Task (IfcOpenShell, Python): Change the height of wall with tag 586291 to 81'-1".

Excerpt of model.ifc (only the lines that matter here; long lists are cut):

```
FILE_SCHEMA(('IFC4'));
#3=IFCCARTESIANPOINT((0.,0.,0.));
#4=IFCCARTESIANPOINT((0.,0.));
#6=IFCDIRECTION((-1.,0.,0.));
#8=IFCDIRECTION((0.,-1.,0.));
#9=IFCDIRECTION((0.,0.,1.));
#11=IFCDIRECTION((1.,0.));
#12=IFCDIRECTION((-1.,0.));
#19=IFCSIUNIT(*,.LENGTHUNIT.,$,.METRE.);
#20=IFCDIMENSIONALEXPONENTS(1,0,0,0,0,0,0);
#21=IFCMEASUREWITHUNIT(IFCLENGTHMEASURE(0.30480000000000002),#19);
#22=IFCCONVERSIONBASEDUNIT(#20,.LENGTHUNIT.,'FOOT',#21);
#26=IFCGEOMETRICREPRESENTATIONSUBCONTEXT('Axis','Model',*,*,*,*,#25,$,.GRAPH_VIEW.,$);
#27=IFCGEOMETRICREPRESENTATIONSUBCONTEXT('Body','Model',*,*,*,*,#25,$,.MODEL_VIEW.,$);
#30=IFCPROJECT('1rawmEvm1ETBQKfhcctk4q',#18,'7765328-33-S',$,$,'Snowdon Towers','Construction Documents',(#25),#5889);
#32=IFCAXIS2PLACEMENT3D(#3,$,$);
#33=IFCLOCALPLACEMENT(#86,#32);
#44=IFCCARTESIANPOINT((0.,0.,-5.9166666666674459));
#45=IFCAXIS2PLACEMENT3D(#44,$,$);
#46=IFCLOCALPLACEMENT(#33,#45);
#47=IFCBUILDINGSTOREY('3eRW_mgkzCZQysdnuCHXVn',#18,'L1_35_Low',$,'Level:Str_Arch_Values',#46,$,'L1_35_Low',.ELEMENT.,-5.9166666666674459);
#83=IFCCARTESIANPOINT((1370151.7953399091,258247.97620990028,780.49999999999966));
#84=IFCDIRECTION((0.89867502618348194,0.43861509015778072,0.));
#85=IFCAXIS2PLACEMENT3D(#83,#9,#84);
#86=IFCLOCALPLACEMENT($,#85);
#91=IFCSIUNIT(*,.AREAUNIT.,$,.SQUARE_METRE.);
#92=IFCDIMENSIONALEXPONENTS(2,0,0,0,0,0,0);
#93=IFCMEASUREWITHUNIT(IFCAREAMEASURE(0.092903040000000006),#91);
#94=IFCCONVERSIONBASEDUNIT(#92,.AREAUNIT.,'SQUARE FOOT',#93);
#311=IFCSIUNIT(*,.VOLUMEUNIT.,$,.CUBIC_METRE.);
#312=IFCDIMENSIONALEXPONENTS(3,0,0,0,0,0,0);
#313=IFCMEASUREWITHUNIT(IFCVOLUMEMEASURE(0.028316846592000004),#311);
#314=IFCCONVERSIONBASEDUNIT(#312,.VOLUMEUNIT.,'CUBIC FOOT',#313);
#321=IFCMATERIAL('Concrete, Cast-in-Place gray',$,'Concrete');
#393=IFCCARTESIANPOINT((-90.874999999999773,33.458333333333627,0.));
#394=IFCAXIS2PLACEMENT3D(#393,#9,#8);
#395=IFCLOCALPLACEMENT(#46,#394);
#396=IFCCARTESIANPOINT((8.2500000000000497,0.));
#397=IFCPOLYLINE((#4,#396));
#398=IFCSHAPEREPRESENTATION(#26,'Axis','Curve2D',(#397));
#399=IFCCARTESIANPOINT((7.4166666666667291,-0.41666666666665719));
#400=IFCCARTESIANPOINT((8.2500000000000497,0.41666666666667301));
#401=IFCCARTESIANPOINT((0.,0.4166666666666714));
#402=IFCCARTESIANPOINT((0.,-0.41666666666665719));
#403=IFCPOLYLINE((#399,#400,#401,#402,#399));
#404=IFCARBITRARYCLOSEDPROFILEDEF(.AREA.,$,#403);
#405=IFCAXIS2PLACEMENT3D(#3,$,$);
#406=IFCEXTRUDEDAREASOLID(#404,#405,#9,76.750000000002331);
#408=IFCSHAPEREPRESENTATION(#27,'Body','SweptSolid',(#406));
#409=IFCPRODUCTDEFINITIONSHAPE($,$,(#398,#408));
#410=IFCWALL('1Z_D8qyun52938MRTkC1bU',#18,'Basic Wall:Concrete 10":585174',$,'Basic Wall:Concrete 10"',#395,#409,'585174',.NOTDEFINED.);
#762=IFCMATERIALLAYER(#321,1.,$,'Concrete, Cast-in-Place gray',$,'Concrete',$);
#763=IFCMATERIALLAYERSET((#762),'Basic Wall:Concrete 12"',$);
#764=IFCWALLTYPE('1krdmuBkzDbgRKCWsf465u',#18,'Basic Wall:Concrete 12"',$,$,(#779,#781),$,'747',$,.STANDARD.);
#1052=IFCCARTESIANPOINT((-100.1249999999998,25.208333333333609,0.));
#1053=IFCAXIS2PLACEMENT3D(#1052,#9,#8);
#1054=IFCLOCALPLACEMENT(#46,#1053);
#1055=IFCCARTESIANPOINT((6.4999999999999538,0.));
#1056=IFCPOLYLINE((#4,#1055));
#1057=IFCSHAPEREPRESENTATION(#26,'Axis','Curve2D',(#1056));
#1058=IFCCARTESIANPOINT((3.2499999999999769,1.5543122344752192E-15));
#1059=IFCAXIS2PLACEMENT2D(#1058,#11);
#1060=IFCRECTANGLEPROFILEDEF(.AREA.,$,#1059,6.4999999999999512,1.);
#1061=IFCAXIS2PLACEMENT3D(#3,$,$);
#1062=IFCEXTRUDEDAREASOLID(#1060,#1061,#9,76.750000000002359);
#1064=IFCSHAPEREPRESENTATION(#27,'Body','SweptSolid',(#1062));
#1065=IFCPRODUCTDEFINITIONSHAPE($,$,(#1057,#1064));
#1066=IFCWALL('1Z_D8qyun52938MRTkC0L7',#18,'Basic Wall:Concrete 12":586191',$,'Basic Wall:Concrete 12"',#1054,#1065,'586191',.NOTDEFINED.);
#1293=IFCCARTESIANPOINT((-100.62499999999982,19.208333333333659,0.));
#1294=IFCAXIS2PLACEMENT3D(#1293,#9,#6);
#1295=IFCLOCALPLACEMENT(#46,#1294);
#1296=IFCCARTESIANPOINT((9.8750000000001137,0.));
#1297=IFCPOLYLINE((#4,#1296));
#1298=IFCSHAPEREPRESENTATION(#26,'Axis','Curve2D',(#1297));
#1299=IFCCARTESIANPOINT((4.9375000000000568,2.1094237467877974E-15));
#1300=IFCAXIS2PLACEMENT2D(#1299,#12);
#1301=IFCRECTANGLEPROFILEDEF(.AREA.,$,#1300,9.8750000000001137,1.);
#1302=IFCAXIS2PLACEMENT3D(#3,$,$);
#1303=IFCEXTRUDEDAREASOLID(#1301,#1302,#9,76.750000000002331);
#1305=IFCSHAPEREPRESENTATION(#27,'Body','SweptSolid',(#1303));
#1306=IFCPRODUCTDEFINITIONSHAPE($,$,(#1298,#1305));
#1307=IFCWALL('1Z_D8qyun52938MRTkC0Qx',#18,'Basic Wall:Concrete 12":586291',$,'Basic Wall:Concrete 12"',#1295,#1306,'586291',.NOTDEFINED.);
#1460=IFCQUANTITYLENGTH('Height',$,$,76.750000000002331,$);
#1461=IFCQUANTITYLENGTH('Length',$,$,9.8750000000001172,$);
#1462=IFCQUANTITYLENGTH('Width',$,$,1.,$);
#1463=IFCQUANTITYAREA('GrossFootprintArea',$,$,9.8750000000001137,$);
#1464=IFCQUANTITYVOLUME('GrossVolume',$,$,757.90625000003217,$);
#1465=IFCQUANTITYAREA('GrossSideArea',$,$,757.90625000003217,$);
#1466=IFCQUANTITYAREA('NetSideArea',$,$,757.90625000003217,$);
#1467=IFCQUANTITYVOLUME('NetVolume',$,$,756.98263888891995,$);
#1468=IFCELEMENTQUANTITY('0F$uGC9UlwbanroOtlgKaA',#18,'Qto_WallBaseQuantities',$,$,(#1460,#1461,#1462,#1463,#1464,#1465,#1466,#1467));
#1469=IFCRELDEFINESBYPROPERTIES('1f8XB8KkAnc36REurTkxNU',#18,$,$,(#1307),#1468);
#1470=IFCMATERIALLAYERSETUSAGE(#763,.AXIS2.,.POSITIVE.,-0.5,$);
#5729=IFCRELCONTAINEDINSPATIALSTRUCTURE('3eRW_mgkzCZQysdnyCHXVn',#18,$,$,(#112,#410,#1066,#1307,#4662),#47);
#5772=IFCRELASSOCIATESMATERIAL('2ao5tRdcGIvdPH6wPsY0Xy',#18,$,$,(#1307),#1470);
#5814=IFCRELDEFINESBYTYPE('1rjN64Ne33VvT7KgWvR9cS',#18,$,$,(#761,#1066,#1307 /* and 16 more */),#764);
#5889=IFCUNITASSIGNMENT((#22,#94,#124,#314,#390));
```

```python
import ifcopenshell
import ifcopenshell.api.pset
import ifcopenshell.geom
import ifcopenshell.util.element
import ifcopenshell.util.representation
import ifcopenshell.util.shape
import ifcopenshell.util.unit

model = ifcopenshell.open("model.ifc")
unit_scale = ifcopenshell.util.unit.calculate_unit_scale(model)
area_scale = ifcopenshell.util.unit.calculate_unit_scale(model, "AREAUNIT")
volume_scale = ifcopenshell.util.unit.calculate_unit_scale(model, "VOLUMEUNIT")
settings = ifcopenshell.geom.settings()


def volume(element):
    """Net volume in cubic metres, openings subtracted."""
    shape = ifcopenshell.geom.create_shape(settings, element)
    return ifcopenshell.util.shape.get_volume(shape.geometry)


wall = model.by_id(1307)
before = volume(wall)

body = ifcopenshell.util.representation.get_representation(wall, "Model", "Body")
solid = body.Items[0]
old_height = solid.Depth
solid.Depth = 973 * 0.0254 / unit_scale
after = volume(wall)
thickness = 0.3048  # wall thickness in metres

# Update the stored height, areas and volumes.
qto = model.by_id(ifcopenshell.util.element.get_pset(wall, "Qto_WallBaseQuantities", should_inherit=False)["id"])
ifcopenshell.api.pset.edit_qto(model, qto=qto, properties={
    "Height": solid.Depth,
    "GrossVolume": ifcopenshell.util.element.get_pset(wall, "Qto_WallBaseQuantities", "GrossVolume") * solid.Depth / old_height,
    "GrossSideArea": ifcopenshell.util.element.get_pset(wall, "Qto_WallBaseQuantities", "GrossSideArea") * solid.Depth / old_height,
    "NetSideArea": after / thickness / area_scale,
    "NetVolume": after / volume_scale,
})

print(f"height {old_height:g} -> {solid.Depth:g}, volume {before:.3f} -> {after:.3f} m3")

model.write("model_updated.ifc")
```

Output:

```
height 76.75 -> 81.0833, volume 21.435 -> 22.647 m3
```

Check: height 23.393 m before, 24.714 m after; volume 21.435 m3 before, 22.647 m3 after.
